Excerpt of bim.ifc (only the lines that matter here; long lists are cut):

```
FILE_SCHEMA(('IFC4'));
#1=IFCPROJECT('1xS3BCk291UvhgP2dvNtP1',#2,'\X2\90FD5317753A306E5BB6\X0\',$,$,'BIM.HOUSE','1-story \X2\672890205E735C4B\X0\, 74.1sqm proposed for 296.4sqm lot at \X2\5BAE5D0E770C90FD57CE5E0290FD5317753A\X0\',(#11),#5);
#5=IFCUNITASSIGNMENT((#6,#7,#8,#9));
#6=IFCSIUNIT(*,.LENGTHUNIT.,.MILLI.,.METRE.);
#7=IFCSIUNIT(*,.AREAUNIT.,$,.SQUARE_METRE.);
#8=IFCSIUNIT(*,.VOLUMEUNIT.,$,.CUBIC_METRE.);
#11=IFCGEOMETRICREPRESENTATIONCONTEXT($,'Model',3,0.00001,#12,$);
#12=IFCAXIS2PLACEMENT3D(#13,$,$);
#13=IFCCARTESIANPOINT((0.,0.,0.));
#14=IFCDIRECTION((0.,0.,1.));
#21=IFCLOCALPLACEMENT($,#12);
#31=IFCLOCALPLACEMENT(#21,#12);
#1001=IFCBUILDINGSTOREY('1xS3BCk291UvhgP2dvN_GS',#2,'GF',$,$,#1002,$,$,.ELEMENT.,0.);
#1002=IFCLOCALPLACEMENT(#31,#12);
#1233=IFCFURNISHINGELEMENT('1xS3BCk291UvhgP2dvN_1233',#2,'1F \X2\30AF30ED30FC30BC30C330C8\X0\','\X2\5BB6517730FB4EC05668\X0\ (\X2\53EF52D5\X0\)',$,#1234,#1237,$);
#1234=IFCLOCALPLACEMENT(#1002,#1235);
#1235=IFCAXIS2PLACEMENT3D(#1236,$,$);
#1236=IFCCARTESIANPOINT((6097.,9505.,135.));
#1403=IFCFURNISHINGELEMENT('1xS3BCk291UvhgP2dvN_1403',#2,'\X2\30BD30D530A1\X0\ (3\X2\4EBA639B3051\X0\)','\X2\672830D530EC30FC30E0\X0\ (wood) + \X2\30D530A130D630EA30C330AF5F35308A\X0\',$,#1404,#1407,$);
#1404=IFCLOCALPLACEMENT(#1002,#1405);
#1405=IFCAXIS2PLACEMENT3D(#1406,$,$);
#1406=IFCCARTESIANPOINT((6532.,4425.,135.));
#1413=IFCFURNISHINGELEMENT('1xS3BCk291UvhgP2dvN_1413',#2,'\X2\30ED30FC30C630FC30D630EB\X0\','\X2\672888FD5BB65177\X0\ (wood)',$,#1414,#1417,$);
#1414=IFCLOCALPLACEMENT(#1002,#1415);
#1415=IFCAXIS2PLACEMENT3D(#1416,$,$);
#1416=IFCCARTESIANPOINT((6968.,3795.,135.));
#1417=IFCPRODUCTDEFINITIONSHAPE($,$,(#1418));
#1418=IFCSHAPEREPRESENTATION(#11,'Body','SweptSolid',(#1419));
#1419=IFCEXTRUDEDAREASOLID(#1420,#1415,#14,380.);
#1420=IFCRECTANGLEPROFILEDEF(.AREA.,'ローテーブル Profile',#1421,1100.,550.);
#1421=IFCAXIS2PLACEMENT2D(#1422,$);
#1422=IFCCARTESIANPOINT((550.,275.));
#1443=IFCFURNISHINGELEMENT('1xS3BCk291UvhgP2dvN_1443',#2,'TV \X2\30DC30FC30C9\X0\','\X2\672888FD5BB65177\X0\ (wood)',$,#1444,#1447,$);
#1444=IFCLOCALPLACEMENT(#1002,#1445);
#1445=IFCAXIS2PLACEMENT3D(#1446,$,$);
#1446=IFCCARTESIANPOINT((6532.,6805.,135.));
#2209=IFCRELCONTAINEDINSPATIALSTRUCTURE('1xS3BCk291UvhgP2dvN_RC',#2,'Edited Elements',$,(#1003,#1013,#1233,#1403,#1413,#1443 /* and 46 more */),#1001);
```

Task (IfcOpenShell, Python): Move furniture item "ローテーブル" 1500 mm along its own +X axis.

```python
import ifcopenshell
import ifcopenshell.api.geometry
import ifcopenshell.util.placement
import ifcopenshell.util.unit

model = ifcopenshell.open("bim.ifc")
unit_scale = ifcopenshell.util.unit.calculate_unit_scale(model)

item = model.by_guid("1xS3BCk291UvhgP2dvN_1413")
matrix = ifcopenshell.util.placement.get_local_placement(item.ObjectPlacement)
matrix[:3, 3] += matrix[:3, 0] * 1.5 / unit_scale
ifcopenshell.api.geometry.edit_object_placement(model, product=item, matrix=matrix, is_si=False)

print(ifcopenshell.util.placement.get_local_placement(item.ObjectPlacement).round(3) + 0.0)

model.write("bim_rev.ifc")
```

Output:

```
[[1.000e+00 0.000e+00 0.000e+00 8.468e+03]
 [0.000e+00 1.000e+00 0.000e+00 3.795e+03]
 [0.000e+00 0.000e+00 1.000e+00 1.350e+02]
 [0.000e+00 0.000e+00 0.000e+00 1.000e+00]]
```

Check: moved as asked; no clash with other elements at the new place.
